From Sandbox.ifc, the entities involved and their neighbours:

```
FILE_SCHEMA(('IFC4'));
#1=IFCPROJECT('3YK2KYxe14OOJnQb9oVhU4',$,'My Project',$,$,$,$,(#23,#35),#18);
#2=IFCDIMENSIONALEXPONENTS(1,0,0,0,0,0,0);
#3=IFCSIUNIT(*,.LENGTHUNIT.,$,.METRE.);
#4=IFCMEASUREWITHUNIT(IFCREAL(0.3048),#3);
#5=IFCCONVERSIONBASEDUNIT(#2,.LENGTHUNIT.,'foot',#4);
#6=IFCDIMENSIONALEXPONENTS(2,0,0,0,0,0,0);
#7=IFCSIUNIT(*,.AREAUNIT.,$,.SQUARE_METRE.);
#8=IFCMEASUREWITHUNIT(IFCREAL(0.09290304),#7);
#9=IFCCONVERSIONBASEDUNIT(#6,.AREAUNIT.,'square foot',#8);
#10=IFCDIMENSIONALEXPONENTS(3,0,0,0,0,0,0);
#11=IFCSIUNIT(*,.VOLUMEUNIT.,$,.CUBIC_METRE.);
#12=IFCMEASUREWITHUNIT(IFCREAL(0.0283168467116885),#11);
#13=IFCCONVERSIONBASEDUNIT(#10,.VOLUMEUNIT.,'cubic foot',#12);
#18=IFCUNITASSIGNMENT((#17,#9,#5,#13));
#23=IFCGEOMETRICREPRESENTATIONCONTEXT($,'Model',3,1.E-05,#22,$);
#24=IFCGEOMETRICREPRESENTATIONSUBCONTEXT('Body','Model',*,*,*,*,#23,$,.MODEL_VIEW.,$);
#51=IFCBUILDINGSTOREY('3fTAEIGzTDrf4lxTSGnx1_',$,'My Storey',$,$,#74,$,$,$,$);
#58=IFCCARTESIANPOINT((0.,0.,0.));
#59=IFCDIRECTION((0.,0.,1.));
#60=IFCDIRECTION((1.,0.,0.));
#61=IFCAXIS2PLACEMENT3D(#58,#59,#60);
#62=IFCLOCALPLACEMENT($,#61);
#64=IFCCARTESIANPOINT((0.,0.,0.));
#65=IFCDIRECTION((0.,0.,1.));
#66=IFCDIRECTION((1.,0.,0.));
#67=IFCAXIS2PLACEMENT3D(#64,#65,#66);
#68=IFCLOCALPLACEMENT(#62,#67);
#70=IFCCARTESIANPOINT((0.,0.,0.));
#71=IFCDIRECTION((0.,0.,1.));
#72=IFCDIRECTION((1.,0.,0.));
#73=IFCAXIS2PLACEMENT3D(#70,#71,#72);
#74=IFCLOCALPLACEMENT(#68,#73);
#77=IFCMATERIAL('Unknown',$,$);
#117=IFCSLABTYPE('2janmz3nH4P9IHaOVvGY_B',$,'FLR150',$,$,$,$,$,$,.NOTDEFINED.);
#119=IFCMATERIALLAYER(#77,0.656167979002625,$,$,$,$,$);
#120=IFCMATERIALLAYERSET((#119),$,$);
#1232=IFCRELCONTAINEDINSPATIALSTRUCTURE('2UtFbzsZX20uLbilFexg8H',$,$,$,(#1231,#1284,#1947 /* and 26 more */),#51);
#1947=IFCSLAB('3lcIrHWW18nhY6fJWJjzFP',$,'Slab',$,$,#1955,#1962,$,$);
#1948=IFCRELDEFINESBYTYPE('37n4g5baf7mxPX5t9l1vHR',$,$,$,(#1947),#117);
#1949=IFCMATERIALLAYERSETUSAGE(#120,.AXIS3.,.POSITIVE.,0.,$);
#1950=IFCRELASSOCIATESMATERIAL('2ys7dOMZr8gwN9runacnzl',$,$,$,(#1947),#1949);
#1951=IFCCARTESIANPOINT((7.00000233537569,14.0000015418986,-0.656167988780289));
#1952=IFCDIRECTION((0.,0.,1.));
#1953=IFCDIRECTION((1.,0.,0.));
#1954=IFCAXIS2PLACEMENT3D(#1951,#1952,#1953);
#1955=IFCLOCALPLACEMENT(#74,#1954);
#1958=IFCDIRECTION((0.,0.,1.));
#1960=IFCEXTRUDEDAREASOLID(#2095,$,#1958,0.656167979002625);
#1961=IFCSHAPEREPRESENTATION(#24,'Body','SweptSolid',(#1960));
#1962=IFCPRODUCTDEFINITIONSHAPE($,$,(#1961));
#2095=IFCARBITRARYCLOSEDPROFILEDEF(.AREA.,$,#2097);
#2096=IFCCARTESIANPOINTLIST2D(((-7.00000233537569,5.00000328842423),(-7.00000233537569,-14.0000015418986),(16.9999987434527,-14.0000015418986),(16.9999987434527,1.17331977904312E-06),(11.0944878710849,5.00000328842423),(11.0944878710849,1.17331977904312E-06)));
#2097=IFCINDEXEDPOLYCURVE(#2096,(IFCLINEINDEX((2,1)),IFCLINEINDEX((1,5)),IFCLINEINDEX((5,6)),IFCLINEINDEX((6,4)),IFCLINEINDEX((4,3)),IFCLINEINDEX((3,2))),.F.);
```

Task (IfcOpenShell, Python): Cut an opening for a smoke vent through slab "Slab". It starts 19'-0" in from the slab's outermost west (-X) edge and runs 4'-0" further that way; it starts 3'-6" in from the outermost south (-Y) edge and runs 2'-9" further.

```python
import numpy as np
import ifcopenshell
import ifcopenshell.api.feature
import ifcopenshell.api.geometry
import ifcopenshell.api.root
import ifcopenshell.geom
import ifcopenshell.util.placement
import ifcopenshell.util.representation
import ifcopenshell.util.shape
import ifcopenshell.util.unit

model = ifcopenshell.open("Sandbox.ifc")
unit_scale = ifcopenshell.util.unit.calculate_unit_scale(model)
settings = ifcopenshell.geom.settings()


def volume(element):
    """Net volume in cubic metres, openings subtracted."""
    shape = ifcopenshell.geom.create_shape(settings, element)
    return ifcopenshell.util.shape.get_volume(shape.geometry)


slab = model.by_guid("3lcIrHWW18nhY6fJWJjzFP")
before = volume(slab)

# Extent in the slab's own axes, in metres. The edges named are its -X and -Y sides.
slab_shape = ifcopenshell.geom.create_shape(settings, slab)
vertices = ifcopenshell.util.shape.get_vertices(slab_shape.geometry)
x_min, y_min, bottom = vertices.min(axis=0)
top = vertices[:, 2].max()

opening = ifcopenshell.api.root.create_entity(model, ifc_class="IfcOpeningElement", name="Smoke vent opening", predefined_type="OPENING")
context = ifcopenshell.util.representation.get_context(model, "Model", "Body", "MODEL_VIEW")
width, depth = 1.2192, 0.8382
outline = [(0.0, 0.0), (width, 0.0), (width, depth), (0.0, depth), (0.0, 0.0)]
# Overshoot both faces by 50 mm so the cut is clean.
shape = ifcopenshell.api.geometry.add_slab_representation(
    model, context=context, depth=top - bottom + 0.1, polyline=outline
)
ifcopenshell.api.geometry.assign_representation(model, product=opening, representation=shape)

matrix = ifcopenshell.util.placement.get_local_placement(slab.ObjectPlacement)
matrix[:, 3] = matrix @ np.append(np.array([x_min + 5.7912, y_min + 1.0668, bottom - 0.05]) / unit_scale, 1.0)
ifcopenshell.api.geometry.edit_object_placement(model, product=opening, matrix=matrix, is_si=False)
ifcopenshell.api.feature.add_feature(model, feature=opening, element=slab)

after = volume(slab)

print(f"slab volume {before:.3f} -> {after:.3f} m3")

model.write("Sandbox_updated.ifc")
```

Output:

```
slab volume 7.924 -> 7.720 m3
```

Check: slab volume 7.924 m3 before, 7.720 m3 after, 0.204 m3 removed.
